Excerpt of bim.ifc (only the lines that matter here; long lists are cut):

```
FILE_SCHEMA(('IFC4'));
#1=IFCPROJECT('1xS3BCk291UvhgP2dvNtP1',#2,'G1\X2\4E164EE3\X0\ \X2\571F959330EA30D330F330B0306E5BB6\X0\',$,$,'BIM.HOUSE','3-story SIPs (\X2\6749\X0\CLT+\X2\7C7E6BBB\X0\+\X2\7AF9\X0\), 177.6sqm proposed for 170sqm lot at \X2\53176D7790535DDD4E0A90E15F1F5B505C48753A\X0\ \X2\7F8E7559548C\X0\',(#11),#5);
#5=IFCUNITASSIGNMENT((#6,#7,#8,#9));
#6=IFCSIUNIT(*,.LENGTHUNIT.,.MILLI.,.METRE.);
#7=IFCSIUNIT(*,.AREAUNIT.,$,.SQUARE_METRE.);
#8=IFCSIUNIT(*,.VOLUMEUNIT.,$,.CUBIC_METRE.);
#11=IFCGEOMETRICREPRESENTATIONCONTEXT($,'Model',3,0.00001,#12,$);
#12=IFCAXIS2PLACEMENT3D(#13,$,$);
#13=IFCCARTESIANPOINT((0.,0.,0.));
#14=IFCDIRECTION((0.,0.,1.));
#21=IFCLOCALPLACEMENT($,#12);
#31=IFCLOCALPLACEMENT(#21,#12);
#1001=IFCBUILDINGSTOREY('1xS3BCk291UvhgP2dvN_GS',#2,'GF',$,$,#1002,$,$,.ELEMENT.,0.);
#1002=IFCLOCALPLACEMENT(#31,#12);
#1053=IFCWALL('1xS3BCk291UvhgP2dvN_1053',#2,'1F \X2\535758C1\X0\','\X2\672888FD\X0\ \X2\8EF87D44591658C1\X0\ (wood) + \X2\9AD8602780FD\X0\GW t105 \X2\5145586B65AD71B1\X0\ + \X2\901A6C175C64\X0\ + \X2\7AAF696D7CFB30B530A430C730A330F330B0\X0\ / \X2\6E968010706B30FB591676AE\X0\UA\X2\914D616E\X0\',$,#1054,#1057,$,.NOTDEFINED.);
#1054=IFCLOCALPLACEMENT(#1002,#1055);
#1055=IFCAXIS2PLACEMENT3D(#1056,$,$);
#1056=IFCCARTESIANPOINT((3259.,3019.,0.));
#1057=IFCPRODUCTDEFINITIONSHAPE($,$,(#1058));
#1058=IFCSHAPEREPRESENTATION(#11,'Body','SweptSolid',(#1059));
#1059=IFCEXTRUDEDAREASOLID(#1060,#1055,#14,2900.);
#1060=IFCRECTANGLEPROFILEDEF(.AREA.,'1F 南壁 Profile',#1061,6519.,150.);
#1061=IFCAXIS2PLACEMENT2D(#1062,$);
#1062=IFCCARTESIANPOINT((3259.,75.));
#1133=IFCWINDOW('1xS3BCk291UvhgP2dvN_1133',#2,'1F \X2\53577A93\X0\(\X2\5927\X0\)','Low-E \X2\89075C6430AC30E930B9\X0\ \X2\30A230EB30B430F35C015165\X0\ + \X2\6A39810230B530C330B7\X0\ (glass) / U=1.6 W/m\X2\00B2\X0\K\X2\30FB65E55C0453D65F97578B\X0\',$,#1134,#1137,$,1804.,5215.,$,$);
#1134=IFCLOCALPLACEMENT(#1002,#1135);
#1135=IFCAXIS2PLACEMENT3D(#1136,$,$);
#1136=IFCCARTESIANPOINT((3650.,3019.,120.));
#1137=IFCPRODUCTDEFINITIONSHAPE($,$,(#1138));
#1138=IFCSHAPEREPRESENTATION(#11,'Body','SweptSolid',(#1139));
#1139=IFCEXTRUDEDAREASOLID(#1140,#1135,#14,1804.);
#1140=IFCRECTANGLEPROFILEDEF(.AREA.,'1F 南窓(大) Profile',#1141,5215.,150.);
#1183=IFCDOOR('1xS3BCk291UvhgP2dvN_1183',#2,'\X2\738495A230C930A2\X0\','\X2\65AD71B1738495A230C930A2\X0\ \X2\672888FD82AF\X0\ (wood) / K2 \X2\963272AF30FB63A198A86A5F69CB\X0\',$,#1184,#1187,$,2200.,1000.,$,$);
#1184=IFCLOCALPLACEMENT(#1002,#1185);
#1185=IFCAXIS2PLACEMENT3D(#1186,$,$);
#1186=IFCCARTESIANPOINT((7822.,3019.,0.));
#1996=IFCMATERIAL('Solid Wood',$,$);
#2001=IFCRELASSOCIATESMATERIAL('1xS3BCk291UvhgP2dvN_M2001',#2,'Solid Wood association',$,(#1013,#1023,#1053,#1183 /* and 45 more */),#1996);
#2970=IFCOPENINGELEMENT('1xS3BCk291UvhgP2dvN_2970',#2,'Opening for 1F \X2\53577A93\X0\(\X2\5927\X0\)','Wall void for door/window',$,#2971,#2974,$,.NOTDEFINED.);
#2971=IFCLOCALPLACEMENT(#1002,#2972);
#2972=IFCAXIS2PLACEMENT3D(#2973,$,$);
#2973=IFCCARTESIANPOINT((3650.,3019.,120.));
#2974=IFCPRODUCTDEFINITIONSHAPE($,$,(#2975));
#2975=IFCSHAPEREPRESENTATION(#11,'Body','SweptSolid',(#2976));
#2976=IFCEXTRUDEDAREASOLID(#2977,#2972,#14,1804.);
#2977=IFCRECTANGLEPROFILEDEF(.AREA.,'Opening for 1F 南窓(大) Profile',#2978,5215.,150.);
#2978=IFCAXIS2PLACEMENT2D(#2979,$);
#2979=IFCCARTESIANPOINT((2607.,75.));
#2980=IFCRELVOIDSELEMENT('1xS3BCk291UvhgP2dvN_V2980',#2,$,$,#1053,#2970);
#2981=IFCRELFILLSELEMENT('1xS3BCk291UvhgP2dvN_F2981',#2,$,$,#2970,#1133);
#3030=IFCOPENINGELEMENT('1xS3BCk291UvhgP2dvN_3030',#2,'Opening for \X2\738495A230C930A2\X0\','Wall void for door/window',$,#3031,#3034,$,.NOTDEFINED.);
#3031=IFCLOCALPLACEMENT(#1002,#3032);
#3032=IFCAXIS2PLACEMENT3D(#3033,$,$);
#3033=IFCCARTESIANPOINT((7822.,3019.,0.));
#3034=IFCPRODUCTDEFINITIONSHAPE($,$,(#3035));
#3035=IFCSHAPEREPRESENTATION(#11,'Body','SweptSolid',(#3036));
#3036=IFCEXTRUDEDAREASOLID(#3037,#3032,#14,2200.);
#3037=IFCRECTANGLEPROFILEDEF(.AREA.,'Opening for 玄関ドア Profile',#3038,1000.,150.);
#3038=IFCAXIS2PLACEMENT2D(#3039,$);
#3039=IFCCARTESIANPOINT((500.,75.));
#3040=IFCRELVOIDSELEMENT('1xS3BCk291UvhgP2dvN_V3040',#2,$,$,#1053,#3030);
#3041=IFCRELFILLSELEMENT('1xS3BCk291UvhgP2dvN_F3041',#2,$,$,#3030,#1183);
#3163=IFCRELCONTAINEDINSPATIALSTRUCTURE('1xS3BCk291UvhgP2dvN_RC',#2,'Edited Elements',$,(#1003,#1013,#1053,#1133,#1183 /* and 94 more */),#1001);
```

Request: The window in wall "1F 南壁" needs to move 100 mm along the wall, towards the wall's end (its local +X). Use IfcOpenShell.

```python
import ifcopenshell
import ifcopenshell.api.geometry
import ifcopenshell.util.placement
import ifcopenshell.util.unit

model = ifcopenshell.open("bim.ifc")
unit_scale = ifcopenshell.util.unit.calculate_unit_scale(model)

window = model.by_guid("1xS3BCk291UvhgP2dvN_1133")
opening = window.FillsVoids[0].RelatingOpeningElement
wall = opening.VoidsElements[0].RelatingBuildingElement

wall_matrix = ifcopenshell.util.placement.get_local_placement(wall.ObjectPlacement)
shift = wall_matrix[:3, 0] * 0.1 / unit_scale
before = ifcopenshell.util.placement.get_local_placement(window.ObjectPlacement)[:3, 3].copy()

# The window is not placed relative to its opening, so move both.
for product in (opening, window):
    matrix = ifcopenshell.util.placement.get_local_placement(product.ObjectPlacement)
    matrix[:3, 3] += shift
    ifcopenshell.api.geometry.edit_object_placement(model, product=product, matrix=matrix, is_si=False)

after = ifcopenshell.util.placement.get_local_placement(window.ObjectPlacement)[:3, 3]
print("window moved by", (after - before).round(3) + 0.0)

model.write("bim-out.ifc")
```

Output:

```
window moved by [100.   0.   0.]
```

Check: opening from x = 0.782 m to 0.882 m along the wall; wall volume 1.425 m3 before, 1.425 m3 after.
